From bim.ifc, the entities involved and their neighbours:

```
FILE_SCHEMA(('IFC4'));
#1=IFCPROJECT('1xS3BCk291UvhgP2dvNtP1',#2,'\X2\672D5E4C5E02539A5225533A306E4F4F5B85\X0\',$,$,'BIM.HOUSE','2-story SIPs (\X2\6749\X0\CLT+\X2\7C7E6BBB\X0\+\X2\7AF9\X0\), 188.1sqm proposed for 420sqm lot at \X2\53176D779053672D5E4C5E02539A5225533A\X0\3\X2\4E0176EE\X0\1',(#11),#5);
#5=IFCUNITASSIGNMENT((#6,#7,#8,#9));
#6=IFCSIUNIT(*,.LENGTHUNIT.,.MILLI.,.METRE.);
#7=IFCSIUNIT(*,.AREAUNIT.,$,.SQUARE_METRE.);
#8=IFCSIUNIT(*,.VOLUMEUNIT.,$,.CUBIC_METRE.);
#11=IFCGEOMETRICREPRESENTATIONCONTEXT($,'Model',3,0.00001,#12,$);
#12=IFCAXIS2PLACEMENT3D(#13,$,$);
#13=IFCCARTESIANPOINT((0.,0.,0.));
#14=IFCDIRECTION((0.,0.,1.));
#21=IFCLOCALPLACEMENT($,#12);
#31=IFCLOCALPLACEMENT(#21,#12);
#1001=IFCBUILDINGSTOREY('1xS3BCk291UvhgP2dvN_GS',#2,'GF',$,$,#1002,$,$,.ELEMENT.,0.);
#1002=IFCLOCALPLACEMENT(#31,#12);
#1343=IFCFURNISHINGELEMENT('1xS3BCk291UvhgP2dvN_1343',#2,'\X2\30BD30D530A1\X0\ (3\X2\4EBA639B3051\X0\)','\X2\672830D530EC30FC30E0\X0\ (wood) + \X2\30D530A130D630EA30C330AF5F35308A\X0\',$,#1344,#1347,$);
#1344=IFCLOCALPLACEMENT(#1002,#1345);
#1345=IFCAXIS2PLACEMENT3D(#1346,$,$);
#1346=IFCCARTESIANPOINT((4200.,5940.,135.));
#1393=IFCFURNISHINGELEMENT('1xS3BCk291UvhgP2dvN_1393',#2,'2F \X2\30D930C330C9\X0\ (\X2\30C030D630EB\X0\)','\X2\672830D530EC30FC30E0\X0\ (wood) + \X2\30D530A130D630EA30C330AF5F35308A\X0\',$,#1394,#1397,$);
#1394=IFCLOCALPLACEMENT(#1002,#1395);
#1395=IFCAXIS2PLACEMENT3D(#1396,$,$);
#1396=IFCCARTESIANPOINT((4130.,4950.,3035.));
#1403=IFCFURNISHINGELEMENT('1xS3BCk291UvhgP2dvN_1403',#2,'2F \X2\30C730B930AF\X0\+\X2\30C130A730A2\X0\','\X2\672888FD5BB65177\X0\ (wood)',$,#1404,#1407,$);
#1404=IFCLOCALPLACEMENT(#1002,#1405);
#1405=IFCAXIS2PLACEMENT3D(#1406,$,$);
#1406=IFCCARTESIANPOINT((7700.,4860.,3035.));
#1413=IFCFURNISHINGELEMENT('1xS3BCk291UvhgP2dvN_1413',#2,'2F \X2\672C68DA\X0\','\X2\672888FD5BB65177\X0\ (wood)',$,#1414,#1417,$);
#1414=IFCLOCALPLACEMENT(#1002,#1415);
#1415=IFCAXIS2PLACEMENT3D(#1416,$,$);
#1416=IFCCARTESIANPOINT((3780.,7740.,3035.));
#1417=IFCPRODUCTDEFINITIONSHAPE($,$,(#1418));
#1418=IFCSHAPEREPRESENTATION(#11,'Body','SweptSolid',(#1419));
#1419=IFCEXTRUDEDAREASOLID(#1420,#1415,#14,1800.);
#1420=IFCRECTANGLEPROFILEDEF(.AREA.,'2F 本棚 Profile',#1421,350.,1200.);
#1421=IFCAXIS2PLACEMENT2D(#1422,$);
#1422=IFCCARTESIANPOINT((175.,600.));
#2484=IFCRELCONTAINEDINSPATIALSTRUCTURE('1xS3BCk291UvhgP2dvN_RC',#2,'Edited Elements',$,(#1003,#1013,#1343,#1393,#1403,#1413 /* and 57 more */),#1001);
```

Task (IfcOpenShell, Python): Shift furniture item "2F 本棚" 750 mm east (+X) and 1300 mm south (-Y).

```python
import ifcopenshell
import ifcopenshell.api.geometry
import ifcopenshell.util.placement
import ifcopenshell.util.unit

model = ifcopenshell.open("bim.ifc")
unit_scale = ifcopenshell.util.unit.calculate_unit_scale(model)

item = model.by_guid("1xS3BCk291UvhgP2dvN_1413")
matrix = ifcopenshell.util.placement.get_local_placement(item.ObjectPlacement)
matrix[0, 3] += 0.75 / unit_scale
matrix[1, 3] -= 1.3 / unit_scale
ifcopenshell.api.geometry.edit_object_placement(model, product=item, matrix=matrix, is_si=False)

print(ifcopenshell.util.placement.get_local_placement(item.ObjectPlacement).round(3) + 0.0)

model.write("bim_rev.ifc")
```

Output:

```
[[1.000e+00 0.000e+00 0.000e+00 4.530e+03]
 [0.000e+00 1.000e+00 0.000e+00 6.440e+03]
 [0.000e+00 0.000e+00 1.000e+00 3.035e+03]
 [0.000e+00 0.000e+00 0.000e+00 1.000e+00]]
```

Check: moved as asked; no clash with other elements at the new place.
